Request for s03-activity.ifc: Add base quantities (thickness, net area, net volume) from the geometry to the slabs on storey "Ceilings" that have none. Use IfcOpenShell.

First a look at what the model holds.

```python
import ifcopenshell
import ifcopenshell.util.element
import ifcopenshell.util.unit

model = ifcopenshell.open("s03-activity.ifc")
print(model.schema)
for unit_type in ("LENGTHUNIT", "AREAUNIT", "VOLUMEUNIT"):
    print(unit_type, ifcopenshell.util.unit.calculate_unit_scale(model, unit_type))
storey = next(s for s in model.by_type("IfcBuildingStorey") if s.Name == "Ceilings")
slabs = [e for e in ifcopenshell.util.element.get_decomposition(storey) if e.is_a("IfcSlab")]
for e in sorted(slabs, key=lambda e: e.id()):
    print(e.id(), e.is_a(), e.Name, list(ifcopenshell.util.element.get_psets(e, qtos_only=True)), sep=" | ")
```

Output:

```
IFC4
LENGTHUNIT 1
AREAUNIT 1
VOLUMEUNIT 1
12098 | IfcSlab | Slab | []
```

```python
import ifcopenshell
import ifcopenshell.api.pset
import ifcopenshell.geom
import ifcopenshell.util.element
import ifcopenshell.util.shape
import ifcopenshell.util.unit

model = ifcopenshell.open("s03-activity.ifc")
unit_scale = ifcopenshell.util.unit.calculate_unit_scale(model)
area_scale = ifcopenshell.util.unit.calculate_unit_scale(model, "AREAUNIT")
volume_scale = ifcopenshell.util.unit.calculate_unit_scale(model, "VOLUMEUNIT")
settings = ifcopenshell.geom.settings()

storey = next(s for s in model.by_type("IfcBuildingStorey") if s.Name == "Ceilings")
slabs = [e for e in ifcopenshell.util.element.get_decomposition(storey) if e.is_a("IfcSlab")]

for e in sorted(slabs, key=lambda e: e.id()):
    if ifcopenshell.util.element.get_psets(e, qtos_only=True, should_inherit=False):
        continue
    # Geometry comes back in metres, in the element's own axes.
    shape = ifcopenshell.geom.create_shape(settings, e)
    values = {
        "Width": ifcopenshell.util.shape.get_z(shape.geometry) / unit_scale,
        "NetArea": ifcopenshell.util.shape.get_footprint_area(shape.geometry) / area_scale,
        "NetVolume": ifcopenshell.util.shape.get_volume(shape.geometry) / volume_scale,
    }
    qto = ifcopenshell.api.pset.add_qto(model, product=e, name="Qto_SlabBaseQuantities")
    ifcopenshell.api.pset.edit_qto(model, qto=qto, properties=values)
    print(e.id(), {k: round(v, 3) for k, v in values.items()})

model.write("s03-activity-out.ifc")
```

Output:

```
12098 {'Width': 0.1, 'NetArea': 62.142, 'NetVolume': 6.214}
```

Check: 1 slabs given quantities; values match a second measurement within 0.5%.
